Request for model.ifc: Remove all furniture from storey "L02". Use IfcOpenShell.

First a look at what the model holds.

```python
import ifcopenshell
import ifcopenshell.util.element

model = ifcopenshell.open("model.ifc")
print(model.schema)
storey = next(s for s in model.by_type("IfcBuildingStorey") if s.Name == "L02")
furniture = [e for e in ifcopenshell.util.element.get_decomposition(storey) if e.is_a("IfcFurnishingElement")]
seen = {}
for e in furniture:
    element_type = ifcopenshell.util.element.get_type(e)
    name = element_type.Name if element_type not in (None, e) else None
    seen[name] = seen.get(name, 0) + 1
for name, count in sorted(seen.items(), key=str):
    print(count, "x", name)
```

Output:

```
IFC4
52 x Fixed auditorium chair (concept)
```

```python
import ifcopenshell
import ifcopenshell.api.root
import ifcopenshell.util.element

model = ifcopenshell.open("model.ifc")

storey = next(s for s in model.by_type("IfcBuildingStorey") if s.Name == "L02")
furniture = [e for e in ifcopenshell.util.element.get_decomposition(storey) if e.is_a("IfcFurnishingElement")]

for e in furniture:
    ifcopenshell.api.root.remove_product(model, product=e)
print(len(furniture), "removed")

model.write("model_rev.ifc")
```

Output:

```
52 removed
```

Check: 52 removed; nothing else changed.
